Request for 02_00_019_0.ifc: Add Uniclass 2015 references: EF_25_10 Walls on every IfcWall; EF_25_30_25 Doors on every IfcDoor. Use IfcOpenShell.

First a look at what the model holds.

```python
import ifcopenshell

model = ifcopenshell.open("02_00_019_0.ifc")
print(model.schema)
print("classifications:", [c.Name for c in model.by_type("IfcClassification")])
for ifc_class in ("IfcDoor", "IfcRoof", "IfcStair", "IfcWall", "IfcWindow"):
    print(ifc_class, len(model.by_type(ifc_class)))
```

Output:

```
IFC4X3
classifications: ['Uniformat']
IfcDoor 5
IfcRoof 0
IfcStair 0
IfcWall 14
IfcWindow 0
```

```python
import ifcopenshell
import ifcopenshell.api.classification

model = ifcopenshell.open("02_00_019_0.ifc")

system = ifcopenshell.api.classification.add_classification(model, classification="Uniclass 2015")

codes = {
    "IfcWall": ("EF_25_10", "Walls"),
    "IfcDoor": ("EF_25_30_25", "Doors"),
}
for ifc_class, (code, name) in codes.items():
    products = model.by_type(ifc_class)
    ifcopenshell.api.classification.add_reference(
        model, products=products, classification=system, identification=code, name=name
    )
    print(code, len(products))

model.write("02_00_019_0_rev.ifc")
```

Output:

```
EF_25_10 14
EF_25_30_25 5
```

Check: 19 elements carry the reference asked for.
